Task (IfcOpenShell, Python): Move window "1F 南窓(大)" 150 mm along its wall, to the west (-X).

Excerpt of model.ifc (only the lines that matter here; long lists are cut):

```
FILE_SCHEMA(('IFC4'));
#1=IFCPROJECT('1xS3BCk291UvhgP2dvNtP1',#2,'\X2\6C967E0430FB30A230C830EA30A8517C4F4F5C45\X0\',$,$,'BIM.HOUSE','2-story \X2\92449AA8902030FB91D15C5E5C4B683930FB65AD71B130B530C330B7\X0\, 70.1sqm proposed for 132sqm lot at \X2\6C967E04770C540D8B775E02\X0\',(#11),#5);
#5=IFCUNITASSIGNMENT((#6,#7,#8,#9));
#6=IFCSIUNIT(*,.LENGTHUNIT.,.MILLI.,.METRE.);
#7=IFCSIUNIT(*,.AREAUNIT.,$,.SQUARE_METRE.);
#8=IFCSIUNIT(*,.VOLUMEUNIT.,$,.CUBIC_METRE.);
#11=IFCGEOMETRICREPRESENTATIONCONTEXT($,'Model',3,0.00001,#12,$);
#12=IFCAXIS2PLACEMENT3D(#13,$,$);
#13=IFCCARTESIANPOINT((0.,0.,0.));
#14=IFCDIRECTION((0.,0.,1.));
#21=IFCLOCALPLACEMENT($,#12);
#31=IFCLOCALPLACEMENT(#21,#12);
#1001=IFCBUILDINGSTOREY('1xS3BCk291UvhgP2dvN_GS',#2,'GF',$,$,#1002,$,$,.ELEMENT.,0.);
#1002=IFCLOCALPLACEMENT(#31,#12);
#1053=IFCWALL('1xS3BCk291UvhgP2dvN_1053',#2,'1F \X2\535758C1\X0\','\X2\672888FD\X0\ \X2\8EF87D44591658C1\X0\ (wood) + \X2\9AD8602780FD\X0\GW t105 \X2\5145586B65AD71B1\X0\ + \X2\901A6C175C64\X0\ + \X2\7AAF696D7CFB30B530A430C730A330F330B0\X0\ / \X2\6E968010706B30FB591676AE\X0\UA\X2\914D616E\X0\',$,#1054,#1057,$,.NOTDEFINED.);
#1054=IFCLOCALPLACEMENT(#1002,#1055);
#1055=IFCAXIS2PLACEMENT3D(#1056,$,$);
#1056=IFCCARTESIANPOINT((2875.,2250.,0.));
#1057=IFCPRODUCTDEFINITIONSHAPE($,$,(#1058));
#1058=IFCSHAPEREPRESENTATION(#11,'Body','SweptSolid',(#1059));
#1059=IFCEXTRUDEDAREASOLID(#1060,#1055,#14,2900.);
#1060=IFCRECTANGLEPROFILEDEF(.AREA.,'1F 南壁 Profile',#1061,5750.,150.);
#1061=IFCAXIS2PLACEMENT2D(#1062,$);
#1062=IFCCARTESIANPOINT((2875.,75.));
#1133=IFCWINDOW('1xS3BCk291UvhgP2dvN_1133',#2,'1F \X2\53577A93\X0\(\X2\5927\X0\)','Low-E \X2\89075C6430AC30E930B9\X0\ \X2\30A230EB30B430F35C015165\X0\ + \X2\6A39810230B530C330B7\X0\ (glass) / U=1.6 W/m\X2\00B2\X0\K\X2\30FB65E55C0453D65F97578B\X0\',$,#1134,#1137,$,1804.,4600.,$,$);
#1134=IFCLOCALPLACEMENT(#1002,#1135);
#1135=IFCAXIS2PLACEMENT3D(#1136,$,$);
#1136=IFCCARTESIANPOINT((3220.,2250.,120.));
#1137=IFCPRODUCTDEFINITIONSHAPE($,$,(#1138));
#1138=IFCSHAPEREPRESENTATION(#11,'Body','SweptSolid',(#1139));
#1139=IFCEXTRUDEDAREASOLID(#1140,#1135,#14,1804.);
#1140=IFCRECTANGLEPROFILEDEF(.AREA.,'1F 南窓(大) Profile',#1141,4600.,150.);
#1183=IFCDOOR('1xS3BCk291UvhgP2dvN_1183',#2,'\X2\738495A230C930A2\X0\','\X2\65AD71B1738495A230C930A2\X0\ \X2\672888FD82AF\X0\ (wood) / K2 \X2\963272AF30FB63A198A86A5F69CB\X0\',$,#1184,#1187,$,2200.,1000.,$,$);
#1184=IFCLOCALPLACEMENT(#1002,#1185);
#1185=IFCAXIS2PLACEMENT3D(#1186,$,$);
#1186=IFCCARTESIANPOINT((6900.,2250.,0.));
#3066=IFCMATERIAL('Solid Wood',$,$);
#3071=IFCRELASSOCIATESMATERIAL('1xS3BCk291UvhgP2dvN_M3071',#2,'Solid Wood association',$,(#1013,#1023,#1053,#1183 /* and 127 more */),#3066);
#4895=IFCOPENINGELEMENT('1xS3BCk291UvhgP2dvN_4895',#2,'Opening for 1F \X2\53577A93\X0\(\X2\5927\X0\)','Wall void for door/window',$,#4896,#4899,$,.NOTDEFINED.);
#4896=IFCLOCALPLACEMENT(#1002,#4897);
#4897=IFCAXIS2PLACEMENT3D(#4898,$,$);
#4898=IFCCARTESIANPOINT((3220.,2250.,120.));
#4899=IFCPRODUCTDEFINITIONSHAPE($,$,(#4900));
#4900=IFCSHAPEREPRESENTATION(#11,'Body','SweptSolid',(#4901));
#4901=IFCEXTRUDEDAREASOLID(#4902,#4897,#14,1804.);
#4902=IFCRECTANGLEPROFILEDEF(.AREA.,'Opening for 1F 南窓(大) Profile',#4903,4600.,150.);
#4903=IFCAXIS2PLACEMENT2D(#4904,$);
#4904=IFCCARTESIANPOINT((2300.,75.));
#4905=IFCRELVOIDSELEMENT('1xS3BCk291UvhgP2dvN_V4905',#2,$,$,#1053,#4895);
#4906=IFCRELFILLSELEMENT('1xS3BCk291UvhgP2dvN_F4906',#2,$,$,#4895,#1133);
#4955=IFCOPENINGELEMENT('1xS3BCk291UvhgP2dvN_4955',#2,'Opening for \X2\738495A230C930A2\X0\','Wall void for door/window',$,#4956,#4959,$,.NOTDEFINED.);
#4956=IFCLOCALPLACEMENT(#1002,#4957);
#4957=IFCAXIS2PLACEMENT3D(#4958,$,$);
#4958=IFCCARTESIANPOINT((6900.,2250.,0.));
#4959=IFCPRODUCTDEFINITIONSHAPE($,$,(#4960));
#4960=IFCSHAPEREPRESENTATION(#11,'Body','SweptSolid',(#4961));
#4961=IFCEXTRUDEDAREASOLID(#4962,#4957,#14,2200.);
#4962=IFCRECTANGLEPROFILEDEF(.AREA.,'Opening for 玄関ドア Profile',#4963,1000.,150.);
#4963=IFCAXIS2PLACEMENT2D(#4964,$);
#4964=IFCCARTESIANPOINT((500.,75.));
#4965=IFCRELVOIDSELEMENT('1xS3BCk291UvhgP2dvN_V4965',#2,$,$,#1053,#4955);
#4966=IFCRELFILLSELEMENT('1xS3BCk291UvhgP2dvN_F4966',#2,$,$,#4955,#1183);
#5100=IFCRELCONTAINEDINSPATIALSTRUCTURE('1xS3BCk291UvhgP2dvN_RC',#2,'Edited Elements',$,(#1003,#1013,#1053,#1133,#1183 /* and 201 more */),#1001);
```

```python
import ifcopenshell
import ifcopenshell.api.geometry
import ifcopenshell.util.placement

model = ifcopenshell.open("model.ifc")

window = model.by_guid("1xS3BCk291UvhgP2dvN_1133")
opening = window.FillsVoids[0].RelatingOpeningElement
wall = opening.VoidsElements[0].RelatingBuildingElement

wall_matrix = ifcopenshell.util.placement.get_local_placement(wall.ObjectPlacement)
shift = wall_matrix[:3, 0] * -150.0
before = ifcopenshell.util.placement.get_local_placement(window.ObjectPlacement)[:3, 3].copy()

# The window is not placed relative to its opening, so move both.
for product in (opening, window):
    matrix = ifcopenshell.util.placement.get_local_placement(product.ObjectPlacement)
    matrix[:3, 3] += shift
    ifcopenshell.api.geometry.edit_object_placement(model, product=product, matrix=matrix, is_si=False)

after = ifcopenshell.util.placement.get_local_placement(window.ObjectPlacement)[:3, 3]
print("window moved by", (after - before).round(3) + 0.0)

model.write("model_updated.ifc")
```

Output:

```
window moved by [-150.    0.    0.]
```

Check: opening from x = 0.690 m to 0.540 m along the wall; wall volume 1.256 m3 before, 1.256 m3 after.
